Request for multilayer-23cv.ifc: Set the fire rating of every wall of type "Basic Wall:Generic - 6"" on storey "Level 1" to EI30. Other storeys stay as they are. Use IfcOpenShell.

First a look at what the model holds.

```python
import ifcopenshell
import ifcopenshell.util.element

model = ifcopenshell.open("multilayer-23cv.ifc")
print(model.schema)
storey = next(s for s in model.by_type("IfcBuildingStorey") if s.Name == "Level 1")
walls = [e for e in ifcopenshell.util.element.get_decomposition(storey) if e.is_a("IfcWall")]
seen = {}
for e in walls:
    element_type = ifcopenshell.util.element.get_type(e)
    key = (element_type.Name if element_type != e and element_type else None, ifcopenshell.util.element.get_pset(e, "Pset_WallCommon", "FireRating"))
    seen[key] = seen.get(key, 0) + 1
for (name, value), count in sorted(seen.items(), key=str):
    print(count, "x", name, "|", value)
```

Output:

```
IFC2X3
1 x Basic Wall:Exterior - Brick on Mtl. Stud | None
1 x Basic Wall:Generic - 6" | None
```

```python
import ifcopenshell
import ifcopenshell.api.pset
import ifcopenshell.util.element

model = ifcopenshell.open("multilayer-23cv.ifc")

storey = next(s for s in model.by_type("IfcBuildingStorey") if s.Name == "Level 1")
walls = [e for e in ifcopenshell.util.element.get_decomposition(storey) if e.is_a("IfcWall")]

count = 0
for e in walls:
    element_type = ifcopenshell.util.element.get_type(e)
    if element_type in (None, e) or element_type.Name != 'Basic Wall:Generic - 6"':
        continue
    # add_pset returns the element's existing set when there is one.
    pset = ifcopenshell.api.pset.add_pset(model, product=e, name="Pset_WallCommon")
    ifcopenshell.api.pset.edit_pset(model, pset=pset, properties={"FireRating": "EI30"})
    count += 1

print(count, "walls updated")

model.write("multilayer-23cv_updated.ifc")
```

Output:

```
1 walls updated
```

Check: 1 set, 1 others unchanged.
